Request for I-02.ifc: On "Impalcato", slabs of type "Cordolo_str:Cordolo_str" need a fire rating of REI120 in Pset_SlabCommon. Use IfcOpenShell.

First a look at what the model holds.

```python
import ifcopenshell
import ifcopenshell.util.element

model = ifcopenshell.open("I-02.ifc")
print(model.schema)
storey = next(s for s in model.by_type("IfcBuildingStorey") if s.Name == "Impalcato")
slabs = [e for e in ifcopenshell.util.element.get_decomposition(storey) if e.is_a("IfcSlab")]
seen = {}
for e in slabs:
    element_type = ifcopenshell.util.element.get_type(e)
    key = (element_type.Name if element_type != e and element_type else None, ifcopenshell.util.element.get_pset(e, "Pset_SlabCommon", "FireRating"))
    seen[key] = seen.get(key, 0) + 1
for (name, value), count in sorted(seen.items(), key=str):
    print(count, "x", name, "|", value)
```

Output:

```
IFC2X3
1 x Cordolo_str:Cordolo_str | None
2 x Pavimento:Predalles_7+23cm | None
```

```python
import ifcopenshell
import ifcopenshell.api.pset
import ifcopenshell.util.element

model = ifcopenshell.open("I-02.ifc")

storey = next(s for s in model.by_type("IfcBuildingStorey") if s.Name == "Impalcato")
slabs = [e for e in ifcopenshell.util.element.get_decomposition(storey) if e.is_a("IfcSlab")]

count = 0
for e in slabs:
    element_type = ifcopenshell.util.element.get_type(e)
    if element_type in (None, e) or element_type.Name != "Cordolo_str:Cordolo_str":
        continue
    # add_pset returns the element's existing set when there is one.
    pset = ifcopenshell.api.pset.add_pset(model, product=e, name="Pset_SlabCommon")
    ifcopenshell.api.pset.edit_pset(model, pset=pset, properties={"FireRating": "REI120"})
    count += 1

print(count, "slabs updated")

model.write("I-02_rev.ifc")
```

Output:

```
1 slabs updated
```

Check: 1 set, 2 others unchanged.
